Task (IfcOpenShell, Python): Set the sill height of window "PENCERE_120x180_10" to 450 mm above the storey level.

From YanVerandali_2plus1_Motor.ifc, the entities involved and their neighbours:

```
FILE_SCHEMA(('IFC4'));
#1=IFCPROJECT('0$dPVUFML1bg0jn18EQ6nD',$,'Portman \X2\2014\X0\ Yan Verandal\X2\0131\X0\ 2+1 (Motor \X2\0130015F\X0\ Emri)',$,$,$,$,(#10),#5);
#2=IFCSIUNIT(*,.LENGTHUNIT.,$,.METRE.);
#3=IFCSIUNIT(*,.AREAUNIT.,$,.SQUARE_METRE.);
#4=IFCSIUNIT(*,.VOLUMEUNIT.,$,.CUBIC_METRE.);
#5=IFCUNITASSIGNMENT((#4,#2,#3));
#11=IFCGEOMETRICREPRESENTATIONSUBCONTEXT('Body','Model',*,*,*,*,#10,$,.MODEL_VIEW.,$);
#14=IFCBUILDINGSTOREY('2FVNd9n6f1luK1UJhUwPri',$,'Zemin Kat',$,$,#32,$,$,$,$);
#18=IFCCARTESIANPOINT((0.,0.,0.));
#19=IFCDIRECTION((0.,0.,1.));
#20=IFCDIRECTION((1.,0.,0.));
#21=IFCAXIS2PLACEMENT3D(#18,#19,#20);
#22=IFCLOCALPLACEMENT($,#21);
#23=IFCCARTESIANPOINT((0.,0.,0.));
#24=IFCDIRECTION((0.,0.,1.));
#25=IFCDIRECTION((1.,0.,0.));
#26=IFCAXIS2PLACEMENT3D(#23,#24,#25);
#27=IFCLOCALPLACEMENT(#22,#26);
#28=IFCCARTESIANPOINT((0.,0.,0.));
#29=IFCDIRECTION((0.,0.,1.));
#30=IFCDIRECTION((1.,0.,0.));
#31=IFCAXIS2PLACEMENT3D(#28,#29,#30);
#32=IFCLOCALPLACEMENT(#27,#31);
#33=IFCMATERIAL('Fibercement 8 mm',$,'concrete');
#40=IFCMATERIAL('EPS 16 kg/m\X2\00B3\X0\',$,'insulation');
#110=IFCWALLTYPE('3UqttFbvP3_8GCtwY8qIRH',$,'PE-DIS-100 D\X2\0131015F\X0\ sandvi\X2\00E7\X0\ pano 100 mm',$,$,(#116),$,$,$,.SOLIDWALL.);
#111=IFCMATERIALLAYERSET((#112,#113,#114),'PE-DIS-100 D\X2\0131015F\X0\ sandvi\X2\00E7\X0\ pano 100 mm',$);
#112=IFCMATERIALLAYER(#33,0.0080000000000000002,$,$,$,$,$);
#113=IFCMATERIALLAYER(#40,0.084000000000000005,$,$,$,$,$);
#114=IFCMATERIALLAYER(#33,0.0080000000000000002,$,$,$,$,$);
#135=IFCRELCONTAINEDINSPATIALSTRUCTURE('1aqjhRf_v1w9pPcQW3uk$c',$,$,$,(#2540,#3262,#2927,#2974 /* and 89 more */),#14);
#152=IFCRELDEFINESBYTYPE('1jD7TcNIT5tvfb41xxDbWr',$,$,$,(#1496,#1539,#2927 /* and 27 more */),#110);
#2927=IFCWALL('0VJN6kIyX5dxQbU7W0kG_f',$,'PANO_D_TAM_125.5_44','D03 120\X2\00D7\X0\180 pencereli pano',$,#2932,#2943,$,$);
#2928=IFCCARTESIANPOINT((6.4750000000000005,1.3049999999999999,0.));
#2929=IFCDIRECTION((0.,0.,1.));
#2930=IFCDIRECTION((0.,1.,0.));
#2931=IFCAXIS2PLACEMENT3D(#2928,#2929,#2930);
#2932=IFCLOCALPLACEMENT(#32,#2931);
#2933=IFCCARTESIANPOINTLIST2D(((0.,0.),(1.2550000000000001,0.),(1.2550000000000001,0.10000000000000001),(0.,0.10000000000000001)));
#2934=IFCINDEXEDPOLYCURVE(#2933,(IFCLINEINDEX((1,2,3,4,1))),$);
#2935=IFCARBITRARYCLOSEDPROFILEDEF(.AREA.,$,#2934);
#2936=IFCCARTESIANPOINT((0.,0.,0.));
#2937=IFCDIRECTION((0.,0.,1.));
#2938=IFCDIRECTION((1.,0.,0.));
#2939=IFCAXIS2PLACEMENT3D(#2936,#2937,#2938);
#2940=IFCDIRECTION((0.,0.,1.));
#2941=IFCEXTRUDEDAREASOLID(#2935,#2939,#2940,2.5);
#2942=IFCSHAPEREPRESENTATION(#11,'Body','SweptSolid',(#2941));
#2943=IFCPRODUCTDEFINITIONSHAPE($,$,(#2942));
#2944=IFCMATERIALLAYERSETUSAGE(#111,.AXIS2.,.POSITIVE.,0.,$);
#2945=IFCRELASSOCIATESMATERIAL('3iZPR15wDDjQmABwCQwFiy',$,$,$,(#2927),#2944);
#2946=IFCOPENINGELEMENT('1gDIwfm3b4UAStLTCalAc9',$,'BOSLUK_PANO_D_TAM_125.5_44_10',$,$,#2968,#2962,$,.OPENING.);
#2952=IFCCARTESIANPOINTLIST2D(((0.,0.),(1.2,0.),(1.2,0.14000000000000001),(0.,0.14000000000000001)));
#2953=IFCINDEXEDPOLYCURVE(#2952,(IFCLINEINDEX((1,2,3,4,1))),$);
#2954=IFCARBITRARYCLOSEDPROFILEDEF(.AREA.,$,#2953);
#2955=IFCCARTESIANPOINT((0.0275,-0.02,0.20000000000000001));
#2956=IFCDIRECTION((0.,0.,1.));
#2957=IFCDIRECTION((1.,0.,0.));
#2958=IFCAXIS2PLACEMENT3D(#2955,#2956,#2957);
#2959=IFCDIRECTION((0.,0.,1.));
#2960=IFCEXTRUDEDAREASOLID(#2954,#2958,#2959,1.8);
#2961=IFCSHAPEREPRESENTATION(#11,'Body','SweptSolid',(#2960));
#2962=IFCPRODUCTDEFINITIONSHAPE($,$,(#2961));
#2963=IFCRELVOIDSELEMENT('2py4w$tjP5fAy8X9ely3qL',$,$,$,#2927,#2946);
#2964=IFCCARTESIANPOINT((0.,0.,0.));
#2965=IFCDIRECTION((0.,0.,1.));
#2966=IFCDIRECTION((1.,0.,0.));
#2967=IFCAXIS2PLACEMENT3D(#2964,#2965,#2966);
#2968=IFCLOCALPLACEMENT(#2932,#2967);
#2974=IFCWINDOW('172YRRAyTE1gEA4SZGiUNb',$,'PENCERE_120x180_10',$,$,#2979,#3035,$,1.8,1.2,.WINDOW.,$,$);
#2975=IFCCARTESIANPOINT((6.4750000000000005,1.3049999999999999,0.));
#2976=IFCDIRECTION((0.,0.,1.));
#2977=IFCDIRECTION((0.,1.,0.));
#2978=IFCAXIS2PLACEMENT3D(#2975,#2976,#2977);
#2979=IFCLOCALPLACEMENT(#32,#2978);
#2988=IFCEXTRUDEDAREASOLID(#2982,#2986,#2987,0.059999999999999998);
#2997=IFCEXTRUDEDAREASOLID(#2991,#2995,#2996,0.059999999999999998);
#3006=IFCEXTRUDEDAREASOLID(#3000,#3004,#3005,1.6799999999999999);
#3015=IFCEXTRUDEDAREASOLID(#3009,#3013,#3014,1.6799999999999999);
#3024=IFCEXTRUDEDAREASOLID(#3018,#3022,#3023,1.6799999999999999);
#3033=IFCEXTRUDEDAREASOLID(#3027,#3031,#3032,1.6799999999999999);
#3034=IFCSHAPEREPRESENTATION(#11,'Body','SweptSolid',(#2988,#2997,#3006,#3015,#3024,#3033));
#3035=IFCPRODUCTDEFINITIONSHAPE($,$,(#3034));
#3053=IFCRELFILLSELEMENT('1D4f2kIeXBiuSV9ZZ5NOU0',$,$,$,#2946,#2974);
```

```python
import numpy as np
import ifcopenshell
import ifcopenshell.api.geometry
import ifcopenshell.geom
import ifcopenshell.util.element
import ifcopenshell.util.placement
import ifcopenshell.util.shape
import ifcopenshell.util.unit

model = ifcopenshell.open("YanVerandali_2plus1_Motor.ifc")
unit_scale = ifcopenshell.util.unit.calculate_unit_scale(model)

window = model.by_guid("172YRRAyTE1gEA4SZGiUNb")
opening = window.FillsVoids[0].RelatingOpeningElement
storey = ifcopenshell.util.element.get_container(window, ifc_class="IfcBuildingStorey")
level = ifcopenshell.util.placement.get_local_placement(storey.ObjectPlacement)[2, 3]

# The opening's origin need not be at the sill, so measure its lowest point.
shape = ifcopenshell.geom.create_shape(ifcopenshell.geom.settings(), opening)
bottom = ifcopenshell.util.shape.get_shape_bottom_elevation(shape, shape.geometry) / unit_scale
dz = level + 0.45 - bottom

shift = np.array([0.0, 0.0, dz])
# The window is not placed relative to its opening, so move both.
for product in (opening, window):
    matrix = ifcopenshell.util.placement.get_local_placement(product.ObjectPlacement)
    matrix[:3, 3] += shift
    ifcopenshell.api.geometry.edit_object_placement(model, product=product, matrix=matrix, is_si=False)

print(f"moved by {dz * unit_scale:+.3f} m")

model.write("YanVerandali_2plus1_Motor_v2.ifc")
```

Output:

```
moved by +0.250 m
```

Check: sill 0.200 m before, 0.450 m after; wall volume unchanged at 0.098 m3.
